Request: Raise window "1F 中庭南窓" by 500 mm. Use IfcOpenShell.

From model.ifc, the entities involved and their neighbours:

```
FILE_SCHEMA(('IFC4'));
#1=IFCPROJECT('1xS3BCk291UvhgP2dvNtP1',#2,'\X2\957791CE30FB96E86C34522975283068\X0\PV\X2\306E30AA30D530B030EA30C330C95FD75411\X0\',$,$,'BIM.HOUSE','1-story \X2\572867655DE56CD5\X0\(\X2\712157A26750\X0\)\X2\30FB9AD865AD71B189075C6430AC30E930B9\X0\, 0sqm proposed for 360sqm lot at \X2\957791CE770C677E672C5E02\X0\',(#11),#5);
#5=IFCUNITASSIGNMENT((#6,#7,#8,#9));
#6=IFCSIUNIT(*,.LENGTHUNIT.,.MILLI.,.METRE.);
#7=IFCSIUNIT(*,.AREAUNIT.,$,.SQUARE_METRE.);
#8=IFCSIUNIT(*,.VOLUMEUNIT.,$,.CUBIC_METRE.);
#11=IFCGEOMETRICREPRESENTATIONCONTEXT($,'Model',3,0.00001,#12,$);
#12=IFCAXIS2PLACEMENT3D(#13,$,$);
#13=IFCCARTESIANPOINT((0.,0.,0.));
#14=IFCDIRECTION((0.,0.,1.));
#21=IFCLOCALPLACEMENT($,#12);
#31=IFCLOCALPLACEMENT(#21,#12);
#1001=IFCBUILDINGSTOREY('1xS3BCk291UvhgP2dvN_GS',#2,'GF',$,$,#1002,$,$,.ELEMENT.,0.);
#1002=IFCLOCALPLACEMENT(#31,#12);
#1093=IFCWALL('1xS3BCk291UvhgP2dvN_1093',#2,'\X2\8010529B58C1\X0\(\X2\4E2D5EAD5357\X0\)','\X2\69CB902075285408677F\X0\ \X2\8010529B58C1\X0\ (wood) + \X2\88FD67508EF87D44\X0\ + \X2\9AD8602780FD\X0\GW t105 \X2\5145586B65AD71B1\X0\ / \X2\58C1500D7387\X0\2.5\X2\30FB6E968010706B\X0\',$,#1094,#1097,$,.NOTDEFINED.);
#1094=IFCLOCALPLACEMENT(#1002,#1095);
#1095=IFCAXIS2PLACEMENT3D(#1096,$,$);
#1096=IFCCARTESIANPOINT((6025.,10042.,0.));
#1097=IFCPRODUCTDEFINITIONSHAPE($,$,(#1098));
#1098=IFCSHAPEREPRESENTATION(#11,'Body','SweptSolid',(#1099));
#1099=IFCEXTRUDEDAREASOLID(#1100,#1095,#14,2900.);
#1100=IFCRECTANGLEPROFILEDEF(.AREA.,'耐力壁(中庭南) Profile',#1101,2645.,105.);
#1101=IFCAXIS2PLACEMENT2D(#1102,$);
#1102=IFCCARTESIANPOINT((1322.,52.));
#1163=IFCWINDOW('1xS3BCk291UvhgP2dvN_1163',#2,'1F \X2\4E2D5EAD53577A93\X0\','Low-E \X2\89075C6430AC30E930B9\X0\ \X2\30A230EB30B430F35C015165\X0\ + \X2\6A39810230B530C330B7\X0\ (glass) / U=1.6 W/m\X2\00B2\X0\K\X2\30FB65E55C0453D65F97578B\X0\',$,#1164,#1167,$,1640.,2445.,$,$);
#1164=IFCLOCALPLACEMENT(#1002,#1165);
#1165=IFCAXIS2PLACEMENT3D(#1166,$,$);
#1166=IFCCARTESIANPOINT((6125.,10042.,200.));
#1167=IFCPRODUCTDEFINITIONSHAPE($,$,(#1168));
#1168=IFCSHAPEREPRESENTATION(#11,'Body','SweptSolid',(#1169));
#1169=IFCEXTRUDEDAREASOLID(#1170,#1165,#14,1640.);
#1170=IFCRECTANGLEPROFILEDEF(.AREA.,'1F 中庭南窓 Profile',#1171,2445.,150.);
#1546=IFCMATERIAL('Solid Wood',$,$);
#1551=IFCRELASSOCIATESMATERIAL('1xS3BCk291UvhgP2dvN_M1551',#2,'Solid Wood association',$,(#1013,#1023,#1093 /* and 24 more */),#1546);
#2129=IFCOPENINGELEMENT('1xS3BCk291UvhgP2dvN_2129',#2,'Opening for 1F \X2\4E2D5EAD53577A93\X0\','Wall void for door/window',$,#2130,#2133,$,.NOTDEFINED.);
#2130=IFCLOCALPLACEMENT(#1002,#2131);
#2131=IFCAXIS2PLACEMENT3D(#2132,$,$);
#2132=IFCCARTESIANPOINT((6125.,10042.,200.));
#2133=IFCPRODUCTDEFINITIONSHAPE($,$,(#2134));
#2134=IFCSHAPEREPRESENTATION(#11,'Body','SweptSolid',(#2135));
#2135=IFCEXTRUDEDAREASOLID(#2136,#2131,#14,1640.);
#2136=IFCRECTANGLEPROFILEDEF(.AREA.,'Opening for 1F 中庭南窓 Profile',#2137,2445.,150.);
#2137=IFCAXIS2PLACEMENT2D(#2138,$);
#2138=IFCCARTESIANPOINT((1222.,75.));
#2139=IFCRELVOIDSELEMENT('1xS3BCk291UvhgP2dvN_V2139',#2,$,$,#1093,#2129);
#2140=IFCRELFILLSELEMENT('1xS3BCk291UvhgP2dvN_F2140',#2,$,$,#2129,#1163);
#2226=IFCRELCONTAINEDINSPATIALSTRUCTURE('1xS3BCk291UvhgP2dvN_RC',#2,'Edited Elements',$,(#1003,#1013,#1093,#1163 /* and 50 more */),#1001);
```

```python
import numpy as np
import ifcopenshell
import ifcopenshell.api.geometry
import ifcopenshell.util.placement
import ifcopenshell.util.unit

model = ifcopenshell.open("model.ifc")
unit_scale = ifcopenshell.util.unit.calculate_unit_scale(model)

window = model.by_guid("1xS3BCk291UvhgP2dvN_1163")
opening = window.FillsVoids[0].RelatingOpeningElement
dz = 0.5 / unit_scale

shift = np.array([0.0, 0.0, dz])
# The window is not placed relative to its opening, so move both.
for product in (opening, window):
    matrix = ifcopenshell.util.placement.get_local_placement(product.ObjectPlacement)
    matrix[:3, 3] += shift
    ifcopenshell.api.geometry.edit_object_placement(model, product=product, matrix=matrix, is_si=False)

print(f"moved by {dz * unit_scale:+.3f} m")

model.write("model_rev.ifc")
```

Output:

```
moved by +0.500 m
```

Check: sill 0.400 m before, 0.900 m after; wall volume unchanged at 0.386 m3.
